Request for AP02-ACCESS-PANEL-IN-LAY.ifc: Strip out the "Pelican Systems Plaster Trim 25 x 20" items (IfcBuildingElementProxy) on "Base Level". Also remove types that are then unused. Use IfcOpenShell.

First a look at what the model holds.

```python
import ifcopenshell
import ifcopenshell.util.element

model = ifcopenshell.open("AP02-ACCESS-PANEL-IN-LAY.ifc")
print(model.schema)
storey = next(s for s in model.by_type("IfcBuildingStorey") if s.Name == "Base Level")
proxies = [e for e in ifcopenshell.util.element.get_decomposition(storey) if e.is_a("IfcBuildingElementProxy")]
seen = {}
for e in proxies:
    element_type = ifcopenshell.util.element.get_type(e)
    name = element_type.Name if element_type not in (None, e) else None
    seen[name] = seen.get(name, 0) + 1
for name, count in sorted(seen.items(), key=str):
    print(count, "x", name)
```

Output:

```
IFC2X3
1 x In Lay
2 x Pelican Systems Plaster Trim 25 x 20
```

```python
import ifcopenshell
import ifcopenshell.api.root
import ifcopenshell.util.element

model = ifcopenshell.open("AP02-ACCESS-PANEL-IN-LAY.ifc")

storey = next(s for s in model.by_type("IfcBuildingStorey") if s.Name == "Base Level")
proxies = [e for e in ifcopenshell.util.element.get_decomposition(storey) if e.is_a("IfcBuildingElementProxy")]
targets = [e for e in proxies if (t := ifcopenshell.util.element.get_type(e)) not in (None, e) and t.Name == "Pelican Systems Plaster Trim 25 x 20"]
types = {ifcopenshell.util.element.get_type(e) for e in targets} - {None, *targets}

for e in targets:
    ifcopenshell.api.root.remove_product(model, product=e)
print(len(targets), "removed")

unused = [t for t in types if not ifcopenshell.util.element.get_types(t)]
for t in unused:
    ifcopenshell.api.root.remove_product(model, product=t)
print(len(unused), "unused types removed")

model.write("AP02-ACCESS-PANEL-IN-LAY_edited.ifc")
```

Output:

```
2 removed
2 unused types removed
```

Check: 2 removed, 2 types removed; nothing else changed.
